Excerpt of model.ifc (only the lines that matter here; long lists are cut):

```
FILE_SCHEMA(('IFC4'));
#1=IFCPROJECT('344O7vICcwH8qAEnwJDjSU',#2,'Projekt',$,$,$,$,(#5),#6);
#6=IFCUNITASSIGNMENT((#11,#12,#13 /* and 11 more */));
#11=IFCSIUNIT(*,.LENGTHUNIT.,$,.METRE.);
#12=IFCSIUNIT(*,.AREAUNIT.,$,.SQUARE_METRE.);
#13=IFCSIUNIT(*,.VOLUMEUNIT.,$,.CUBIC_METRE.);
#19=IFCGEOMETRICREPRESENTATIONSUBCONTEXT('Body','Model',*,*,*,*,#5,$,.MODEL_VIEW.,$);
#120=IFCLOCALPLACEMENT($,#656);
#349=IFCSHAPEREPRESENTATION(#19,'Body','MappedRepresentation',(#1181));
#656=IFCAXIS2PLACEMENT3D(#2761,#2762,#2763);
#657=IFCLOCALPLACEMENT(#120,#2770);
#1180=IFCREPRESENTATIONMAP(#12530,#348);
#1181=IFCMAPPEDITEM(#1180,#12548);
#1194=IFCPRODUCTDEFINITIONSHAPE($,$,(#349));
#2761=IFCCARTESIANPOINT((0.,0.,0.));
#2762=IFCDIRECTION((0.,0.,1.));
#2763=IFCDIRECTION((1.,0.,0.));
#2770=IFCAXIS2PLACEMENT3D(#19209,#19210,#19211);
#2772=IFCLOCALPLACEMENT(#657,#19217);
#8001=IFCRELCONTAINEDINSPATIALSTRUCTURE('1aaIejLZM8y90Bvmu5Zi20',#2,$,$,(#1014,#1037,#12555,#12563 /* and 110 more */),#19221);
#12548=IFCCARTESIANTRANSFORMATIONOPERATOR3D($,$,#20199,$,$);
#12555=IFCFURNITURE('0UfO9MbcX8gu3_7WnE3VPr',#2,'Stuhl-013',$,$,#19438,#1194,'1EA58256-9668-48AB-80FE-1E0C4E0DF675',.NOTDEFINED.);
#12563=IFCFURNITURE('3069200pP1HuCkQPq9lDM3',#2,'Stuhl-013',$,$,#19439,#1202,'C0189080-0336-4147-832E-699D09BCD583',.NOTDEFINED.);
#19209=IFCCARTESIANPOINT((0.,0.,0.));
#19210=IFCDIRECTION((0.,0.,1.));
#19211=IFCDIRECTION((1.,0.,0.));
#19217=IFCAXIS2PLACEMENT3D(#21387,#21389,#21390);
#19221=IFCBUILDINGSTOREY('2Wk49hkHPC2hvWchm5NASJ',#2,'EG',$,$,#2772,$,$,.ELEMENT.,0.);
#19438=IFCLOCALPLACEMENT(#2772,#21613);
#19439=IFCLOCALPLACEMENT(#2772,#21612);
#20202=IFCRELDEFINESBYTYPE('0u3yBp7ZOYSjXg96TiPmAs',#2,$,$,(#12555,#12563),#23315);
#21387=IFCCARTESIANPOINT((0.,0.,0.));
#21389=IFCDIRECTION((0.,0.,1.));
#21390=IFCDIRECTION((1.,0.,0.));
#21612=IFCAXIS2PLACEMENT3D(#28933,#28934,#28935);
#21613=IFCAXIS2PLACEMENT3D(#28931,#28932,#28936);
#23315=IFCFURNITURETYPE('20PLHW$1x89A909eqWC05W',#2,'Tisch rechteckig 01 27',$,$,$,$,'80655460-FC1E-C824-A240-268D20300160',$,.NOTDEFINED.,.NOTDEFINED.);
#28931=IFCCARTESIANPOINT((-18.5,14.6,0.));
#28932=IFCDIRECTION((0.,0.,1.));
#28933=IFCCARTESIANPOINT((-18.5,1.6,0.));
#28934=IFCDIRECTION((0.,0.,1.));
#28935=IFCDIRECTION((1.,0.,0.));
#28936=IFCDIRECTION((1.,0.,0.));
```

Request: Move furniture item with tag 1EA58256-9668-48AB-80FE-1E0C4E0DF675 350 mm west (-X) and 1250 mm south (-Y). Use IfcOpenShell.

```python
import ifcopenshell
import ifcopenshell.api.geometry
import ifcopenshell.util.placement
import ifcopenshell.util.unit

model = ifcopenshell.open("model.ifc")
unit_scale = ifcopenshell.util.unit.calculate_unit_scale(model)

item = model.by_id(12555)
matrix = ifcopenshell.util.placement.get_local_placement(item.ObjectPlacement)
matrix[0, 3] -= 0.35 / unit_scale
matrix[1, 3] -= 1.25 / unit_scale
ifcopenshell.api.geometry.edit_object_placement(model, product=item, matrix=matrix, is_si=False)

print(ifcopenshell.util.placement.get_local_placement(item.ObjectPlacement).round(3) + 0.0)

model.write("model_edited.ifc")
```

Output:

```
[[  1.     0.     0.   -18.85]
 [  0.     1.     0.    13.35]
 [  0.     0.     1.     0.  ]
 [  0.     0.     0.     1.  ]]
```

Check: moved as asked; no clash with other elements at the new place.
